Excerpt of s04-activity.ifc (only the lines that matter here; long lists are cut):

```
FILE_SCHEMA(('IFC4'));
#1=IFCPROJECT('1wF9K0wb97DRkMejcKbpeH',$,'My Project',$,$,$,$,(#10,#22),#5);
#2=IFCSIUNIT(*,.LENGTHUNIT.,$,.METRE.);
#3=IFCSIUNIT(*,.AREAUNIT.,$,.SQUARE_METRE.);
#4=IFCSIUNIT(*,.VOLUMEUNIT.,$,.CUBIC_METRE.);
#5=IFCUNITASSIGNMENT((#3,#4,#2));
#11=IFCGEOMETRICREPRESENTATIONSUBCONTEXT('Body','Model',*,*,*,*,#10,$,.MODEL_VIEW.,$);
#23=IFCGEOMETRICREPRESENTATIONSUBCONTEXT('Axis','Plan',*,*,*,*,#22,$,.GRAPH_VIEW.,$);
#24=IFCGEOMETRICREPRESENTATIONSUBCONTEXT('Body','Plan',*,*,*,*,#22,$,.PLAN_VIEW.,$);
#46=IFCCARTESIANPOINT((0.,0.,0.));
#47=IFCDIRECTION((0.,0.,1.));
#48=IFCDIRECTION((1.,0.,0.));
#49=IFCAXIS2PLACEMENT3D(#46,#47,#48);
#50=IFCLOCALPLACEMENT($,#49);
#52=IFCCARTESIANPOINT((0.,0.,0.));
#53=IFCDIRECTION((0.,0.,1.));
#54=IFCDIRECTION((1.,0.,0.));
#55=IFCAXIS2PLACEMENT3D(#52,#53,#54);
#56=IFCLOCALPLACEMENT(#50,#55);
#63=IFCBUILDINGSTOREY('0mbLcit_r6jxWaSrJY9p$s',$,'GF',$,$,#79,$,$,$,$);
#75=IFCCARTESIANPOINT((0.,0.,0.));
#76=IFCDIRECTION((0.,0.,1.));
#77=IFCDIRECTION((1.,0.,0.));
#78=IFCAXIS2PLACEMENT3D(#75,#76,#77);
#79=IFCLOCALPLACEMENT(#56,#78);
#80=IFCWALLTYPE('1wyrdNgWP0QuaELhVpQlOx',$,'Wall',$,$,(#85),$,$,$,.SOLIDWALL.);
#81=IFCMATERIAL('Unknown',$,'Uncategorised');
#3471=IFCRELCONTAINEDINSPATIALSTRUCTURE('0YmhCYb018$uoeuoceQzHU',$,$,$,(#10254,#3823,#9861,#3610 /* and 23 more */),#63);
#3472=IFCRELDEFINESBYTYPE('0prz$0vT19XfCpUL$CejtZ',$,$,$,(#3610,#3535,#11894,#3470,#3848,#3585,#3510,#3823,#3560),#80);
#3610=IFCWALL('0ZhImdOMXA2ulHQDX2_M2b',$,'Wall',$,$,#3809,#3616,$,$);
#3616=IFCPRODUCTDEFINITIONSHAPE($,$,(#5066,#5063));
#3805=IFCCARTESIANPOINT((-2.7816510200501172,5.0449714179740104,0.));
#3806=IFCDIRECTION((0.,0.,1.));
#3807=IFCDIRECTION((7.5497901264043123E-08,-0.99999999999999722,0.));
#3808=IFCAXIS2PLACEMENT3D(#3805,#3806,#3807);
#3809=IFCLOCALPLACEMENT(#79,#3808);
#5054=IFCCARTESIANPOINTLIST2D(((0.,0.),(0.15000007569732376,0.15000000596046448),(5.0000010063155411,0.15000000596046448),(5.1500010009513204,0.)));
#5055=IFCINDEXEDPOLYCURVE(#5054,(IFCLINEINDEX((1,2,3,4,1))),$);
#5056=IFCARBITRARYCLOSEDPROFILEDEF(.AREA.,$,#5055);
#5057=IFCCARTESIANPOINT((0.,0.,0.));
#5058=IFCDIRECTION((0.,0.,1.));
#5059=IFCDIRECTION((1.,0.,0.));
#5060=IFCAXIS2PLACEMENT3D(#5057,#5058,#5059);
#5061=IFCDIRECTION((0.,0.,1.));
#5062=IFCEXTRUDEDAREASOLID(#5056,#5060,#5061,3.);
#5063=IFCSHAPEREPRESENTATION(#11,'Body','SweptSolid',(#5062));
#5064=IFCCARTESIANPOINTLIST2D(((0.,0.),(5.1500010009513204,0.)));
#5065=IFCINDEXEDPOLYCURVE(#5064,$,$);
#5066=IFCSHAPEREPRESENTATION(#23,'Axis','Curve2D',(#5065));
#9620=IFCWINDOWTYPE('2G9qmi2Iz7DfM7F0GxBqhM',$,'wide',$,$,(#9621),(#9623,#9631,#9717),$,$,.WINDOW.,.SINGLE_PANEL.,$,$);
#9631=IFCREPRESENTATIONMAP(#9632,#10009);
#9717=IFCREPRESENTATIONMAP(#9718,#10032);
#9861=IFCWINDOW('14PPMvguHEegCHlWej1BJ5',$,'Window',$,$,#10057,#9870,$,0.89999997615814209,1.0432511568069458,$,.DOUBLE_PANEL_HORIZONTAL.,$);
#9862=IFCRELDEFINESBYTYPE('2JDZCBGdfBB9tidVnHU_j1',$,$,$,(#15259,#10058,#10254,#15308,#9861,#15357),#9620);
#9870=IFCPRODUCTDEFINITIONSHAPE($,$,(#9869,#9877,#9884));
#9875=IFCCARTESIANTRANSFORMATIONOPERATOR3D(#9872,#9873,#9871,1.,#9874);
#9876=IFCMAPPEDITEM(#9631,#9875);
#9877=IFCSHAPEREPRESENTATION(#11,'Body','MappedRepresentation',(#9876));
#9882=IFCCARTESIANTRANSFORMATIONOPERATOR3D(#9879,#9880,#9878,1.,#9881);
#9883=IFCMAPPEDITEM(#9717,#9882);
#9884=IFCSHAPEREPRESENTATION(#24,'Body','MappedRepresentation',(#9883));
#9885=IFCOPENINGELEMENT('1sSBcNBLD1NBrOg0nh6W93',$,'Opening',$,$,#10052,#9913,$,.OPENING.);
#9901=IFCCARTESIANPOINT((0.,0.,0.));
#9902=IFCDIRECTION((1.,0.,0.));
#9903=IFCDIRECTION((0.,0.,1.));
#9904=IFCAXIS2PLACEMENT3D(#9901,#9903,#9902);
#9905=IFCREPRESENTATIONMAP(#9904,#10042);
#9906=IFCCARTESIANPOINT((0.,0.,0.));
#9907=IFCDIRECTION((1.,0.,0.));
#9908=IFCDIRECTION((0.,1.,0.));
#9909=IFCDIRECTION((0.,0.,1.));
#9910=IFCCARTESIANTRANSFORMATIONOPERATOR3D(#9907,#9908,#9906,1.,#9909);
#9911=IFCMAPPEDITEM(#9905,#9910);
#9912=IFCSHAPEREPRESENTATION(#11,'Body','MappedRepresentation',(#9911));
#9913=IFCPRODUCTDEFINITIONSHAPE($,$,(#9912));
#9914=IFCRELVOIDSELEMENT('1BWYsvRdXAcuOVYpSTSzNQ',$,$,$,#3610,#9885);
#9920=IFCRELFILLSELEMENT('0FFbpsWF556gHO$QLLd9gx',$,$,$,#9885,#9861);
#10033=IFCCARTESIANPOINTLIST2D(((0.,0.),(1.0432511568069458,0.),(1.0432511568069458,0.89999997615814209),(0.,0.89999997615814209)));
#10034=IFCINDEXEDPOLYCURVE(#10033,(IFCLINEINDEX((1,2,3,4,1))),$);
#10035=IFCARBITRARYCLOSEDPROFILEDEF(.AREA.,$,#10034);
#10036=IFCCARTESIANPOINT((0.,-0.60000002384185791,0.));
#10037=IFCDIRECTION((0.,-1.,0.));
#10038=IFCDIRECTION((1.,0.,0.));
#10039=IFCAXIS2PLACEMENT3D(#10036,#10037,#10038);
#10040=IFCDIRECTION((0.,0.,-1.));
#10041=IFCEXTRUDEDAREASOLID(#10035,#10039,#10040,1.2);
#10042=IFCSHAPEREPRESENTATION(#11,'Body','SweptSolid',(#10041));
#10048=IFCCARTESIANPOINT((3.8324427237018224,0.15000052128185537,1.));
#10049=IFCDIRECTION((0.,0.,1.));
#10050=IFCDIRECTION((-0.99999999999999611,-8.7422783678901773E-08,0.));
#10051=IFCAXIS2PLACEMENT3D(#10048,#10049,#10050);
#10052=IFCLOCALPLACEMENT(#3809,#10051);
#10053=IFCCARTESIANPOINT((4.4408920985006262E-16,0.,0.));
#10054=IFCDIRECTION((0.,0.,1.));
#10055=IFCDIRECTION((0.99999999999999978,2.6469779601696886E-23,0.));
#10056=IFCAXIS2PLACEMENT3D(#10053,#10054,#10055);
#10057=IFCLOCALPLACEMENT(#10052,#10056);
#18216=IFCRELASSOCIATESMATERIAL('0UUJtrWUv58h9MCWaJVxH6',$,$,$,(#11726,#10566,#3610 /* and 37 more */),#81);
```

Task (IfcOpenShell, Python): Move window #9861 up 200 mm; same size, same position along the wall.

```python
import numpy as np
import ifcopenshell
import ifcopenshell.api.geometry
import ifcopenshell.util.placement
import ifcopenshell.util.unit

model = ifcopenshell.open("s04-activity.ifc")
unit_scale = ifcopenshell.util.unit.calculate_unit_scale(model)

window = model.by_guid("14PPMvguHEegCHlWej1BJ5")
opening = window.FillsVoids[0].RelatingOpeningElement
dz = 0.2 / unit_scale

shift = np.array([0.0, 0.0, dz])
# The window is placed relative to its opening, so it follows when the opening moves.
matrix = ifcopenshell.util.placement.get_local_placement(opening.ObjectPlacement)
matrix[:3, 3] += shift
ifcopenshell.api.geometry.edit_object_placement(
    model, product=opening, matrix=matrix, is_si=False, should_transform_children=True
)

print(f"moved by {dz * unit_scale:+.3f} m")

model.write("s04-activity_rev.ifc")
```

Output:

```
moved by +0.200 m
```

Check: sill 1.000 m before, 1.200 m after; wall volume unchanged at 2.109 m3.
